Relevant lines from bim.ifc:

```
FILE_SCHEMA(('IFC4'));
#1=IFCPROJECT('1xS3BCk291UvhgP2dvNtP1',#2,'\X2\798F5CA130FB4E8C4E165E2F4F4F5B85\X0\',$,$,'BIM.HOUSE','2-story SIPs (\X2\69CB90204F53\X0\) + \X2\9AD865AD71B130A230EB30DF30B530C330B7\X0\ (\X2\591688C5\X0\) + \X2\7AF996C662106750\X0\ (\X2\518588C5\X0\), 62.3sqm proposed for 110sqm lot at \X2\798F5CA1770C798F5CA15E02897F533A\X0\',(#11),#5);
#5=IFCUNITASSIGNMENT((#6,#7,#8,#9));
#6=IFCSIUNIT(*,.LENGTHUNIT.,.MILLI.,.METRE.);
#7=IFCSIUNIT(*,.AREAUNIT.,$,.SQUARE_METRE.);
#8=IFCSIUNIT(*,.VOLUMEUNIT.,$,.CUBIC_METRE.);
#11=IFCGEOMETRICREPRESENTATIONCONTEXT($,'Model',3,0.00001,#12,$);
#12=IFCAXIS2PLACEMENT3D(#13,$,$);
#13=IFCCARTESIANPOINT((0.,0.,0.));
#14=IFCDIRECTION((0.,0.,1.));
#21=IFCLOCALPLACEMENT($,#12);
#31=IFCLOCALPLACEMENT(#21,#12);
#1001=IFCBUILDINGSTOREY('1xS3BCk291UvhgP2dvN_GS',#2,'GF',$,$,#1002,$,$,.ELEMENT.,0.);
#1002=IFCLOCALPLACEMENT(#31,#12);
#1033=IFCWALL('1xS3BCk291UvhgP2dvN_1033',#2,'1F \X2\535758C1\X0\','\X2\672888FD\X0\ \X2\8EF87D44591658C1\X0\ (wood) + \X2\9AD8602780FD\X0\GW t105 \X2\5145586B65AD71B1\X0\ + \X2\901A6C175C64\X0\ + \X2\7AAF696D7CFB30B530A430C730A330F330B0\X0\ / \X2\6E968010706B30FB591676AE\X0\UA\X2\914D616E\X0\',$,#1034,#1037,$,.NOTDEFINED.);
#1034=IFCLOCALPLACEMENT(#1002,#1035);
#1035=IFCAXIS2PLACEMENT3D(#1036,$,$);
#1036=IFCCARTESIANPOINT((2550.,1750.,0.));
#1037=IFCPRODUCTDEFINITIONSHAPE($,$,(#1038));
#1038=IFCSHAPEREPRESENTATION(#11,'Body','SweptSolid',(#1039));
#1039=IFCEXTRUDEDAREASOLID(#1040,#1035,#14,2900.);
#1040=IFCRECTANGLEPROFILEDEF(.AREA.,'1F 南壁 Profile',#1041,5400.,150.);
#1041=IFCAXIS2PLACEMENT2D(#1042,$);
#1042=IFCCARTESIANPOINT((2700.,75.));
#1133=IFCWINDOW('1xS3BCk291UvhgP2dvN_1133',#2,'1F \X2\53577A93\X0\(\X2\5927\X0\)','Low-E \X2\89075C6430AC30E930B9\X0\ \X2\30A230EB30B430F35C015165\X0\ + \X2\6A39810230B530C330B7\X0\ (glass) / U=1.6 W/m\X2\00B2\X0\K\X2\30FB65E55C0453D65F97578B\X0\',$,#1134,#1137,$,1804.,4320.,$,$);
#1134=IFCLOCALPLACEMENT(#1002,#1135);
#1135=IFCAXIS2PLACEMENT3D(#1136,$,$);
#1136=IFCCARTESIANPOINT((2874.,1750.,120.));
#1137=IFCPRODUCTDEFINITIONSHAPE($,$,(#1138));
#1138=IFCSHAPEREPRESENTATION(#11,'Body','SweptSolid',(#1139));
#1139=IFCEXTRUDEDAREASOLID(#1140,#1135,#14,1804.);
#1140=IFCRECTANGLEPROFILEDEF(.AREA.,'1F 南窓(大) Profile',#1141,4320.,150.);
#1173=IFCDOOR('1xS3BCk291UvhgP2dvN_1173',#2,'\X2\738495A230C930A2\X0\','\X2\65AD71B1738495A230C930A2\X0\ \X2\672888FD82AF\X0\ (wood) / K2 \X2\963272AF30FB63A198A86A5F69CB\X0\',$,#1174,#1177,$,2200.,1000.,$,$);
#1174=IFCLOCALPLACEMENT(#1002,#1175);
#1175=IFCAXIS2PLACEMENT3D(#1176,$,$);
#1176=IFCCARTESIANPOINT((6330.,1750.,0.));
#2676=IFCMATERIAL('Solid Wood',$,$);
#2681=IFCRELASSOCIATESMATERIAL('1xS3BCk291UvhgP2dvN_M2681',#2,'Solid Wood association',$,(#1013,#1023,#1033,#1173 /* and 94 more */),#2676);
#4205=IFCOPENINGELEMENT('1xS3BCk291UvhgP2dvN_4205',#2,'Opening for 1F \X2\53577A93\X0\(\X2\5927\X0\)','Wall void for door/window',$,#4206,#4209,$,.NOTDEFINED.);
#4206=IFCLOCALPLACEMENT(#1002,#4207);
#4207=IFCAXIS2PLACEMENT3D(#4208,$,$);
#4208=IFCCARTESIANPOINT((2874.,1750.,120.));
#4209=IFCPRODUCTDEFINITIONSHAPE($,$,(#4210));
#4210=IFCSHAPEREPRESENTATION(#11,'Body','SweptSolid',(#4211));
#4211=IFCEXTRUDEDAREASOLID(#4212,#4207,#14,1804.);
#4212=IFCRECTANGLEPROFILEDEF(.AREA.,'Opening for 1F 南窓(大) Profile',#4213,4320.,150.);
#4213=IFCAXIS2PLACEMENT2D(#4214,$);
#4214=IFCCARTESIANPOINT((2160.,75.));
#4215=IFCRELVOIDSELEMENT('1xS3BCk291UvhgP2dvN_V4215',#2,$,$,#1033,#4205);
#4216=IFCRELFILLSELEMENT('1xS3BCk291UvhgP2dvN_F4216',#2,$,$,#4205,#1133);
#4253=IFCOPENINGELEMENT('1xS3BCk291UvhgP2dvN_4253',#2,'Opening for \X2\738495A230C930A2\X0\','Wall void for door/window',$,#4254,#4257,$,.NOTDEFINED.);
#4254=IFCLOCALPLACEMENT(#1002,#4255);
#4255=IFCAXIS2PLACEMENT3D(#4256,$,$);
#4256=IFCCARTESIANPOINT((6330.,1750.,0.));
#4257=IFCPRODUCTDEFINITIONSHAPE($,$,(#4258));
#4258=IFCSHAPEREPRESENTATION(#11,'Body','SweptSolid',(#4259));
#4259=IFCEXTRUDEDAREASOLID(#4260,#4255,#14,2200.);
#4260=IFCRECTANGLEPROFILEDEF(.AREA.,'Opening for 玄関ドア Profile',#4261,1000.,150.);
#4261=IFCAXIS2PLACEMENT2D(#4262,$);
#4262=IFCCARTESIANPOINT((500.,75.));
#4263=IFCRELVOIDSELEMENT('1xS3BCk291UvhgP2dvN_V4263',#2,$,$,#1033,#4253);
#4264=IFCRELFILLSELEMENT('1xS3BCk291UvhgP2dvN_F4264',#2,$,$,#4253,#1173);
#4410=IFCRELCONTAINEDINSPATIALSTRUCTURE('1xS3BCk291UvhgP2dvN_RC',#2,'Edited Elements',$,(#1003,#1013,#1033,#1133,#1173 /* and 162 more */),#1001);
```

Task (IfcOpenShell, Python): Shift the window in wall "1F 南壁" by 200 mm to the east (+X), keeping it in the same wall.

```python
import ifcopenshell
import ifcopenshell.api.geometry
import ifcopenshell.util.placement

model = ifcopenshell.open("bim.ifc")

window = model.by_guid("1xS3BCk291UvhgP2dvN_1133")
opening = window.FillsVoids[0].RelatingOpeningElement
wall = opening.VoidsElements[0].RelatingBuildingElement

wall_matrix = ifcopenshell.util.placement.get_local_placement(wall.ObjectPlacement)
shift = wall_matrix[:3, 0] * 200.0
before = ifcopenshell.util.placement.get_local_placement(window.ObjectPlacement)[:3, 3].copy()

# The window is not placed relative to its opening, so move both.
for product in (opening, window):
    matrix = ifcopenshell.util.placement.get_local_placement(product.ObjectPlacement)
    matrix[:3, 3] += shift
    ifcopenshell.api.geometry.edit_object_placement(model, product=product, matrix=matrix, is_si=False)

after = ifcopenshell.util.placement.get_local_placement(window.ObjectPlacement)[:3, 3]
print("window moved by", (after - before).round(3) + 0.0)

model.write("bim-out.ifc")
```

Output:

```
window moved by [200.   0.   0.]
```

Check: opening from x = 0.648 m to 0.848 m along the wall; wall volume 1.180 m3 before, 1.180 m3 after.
